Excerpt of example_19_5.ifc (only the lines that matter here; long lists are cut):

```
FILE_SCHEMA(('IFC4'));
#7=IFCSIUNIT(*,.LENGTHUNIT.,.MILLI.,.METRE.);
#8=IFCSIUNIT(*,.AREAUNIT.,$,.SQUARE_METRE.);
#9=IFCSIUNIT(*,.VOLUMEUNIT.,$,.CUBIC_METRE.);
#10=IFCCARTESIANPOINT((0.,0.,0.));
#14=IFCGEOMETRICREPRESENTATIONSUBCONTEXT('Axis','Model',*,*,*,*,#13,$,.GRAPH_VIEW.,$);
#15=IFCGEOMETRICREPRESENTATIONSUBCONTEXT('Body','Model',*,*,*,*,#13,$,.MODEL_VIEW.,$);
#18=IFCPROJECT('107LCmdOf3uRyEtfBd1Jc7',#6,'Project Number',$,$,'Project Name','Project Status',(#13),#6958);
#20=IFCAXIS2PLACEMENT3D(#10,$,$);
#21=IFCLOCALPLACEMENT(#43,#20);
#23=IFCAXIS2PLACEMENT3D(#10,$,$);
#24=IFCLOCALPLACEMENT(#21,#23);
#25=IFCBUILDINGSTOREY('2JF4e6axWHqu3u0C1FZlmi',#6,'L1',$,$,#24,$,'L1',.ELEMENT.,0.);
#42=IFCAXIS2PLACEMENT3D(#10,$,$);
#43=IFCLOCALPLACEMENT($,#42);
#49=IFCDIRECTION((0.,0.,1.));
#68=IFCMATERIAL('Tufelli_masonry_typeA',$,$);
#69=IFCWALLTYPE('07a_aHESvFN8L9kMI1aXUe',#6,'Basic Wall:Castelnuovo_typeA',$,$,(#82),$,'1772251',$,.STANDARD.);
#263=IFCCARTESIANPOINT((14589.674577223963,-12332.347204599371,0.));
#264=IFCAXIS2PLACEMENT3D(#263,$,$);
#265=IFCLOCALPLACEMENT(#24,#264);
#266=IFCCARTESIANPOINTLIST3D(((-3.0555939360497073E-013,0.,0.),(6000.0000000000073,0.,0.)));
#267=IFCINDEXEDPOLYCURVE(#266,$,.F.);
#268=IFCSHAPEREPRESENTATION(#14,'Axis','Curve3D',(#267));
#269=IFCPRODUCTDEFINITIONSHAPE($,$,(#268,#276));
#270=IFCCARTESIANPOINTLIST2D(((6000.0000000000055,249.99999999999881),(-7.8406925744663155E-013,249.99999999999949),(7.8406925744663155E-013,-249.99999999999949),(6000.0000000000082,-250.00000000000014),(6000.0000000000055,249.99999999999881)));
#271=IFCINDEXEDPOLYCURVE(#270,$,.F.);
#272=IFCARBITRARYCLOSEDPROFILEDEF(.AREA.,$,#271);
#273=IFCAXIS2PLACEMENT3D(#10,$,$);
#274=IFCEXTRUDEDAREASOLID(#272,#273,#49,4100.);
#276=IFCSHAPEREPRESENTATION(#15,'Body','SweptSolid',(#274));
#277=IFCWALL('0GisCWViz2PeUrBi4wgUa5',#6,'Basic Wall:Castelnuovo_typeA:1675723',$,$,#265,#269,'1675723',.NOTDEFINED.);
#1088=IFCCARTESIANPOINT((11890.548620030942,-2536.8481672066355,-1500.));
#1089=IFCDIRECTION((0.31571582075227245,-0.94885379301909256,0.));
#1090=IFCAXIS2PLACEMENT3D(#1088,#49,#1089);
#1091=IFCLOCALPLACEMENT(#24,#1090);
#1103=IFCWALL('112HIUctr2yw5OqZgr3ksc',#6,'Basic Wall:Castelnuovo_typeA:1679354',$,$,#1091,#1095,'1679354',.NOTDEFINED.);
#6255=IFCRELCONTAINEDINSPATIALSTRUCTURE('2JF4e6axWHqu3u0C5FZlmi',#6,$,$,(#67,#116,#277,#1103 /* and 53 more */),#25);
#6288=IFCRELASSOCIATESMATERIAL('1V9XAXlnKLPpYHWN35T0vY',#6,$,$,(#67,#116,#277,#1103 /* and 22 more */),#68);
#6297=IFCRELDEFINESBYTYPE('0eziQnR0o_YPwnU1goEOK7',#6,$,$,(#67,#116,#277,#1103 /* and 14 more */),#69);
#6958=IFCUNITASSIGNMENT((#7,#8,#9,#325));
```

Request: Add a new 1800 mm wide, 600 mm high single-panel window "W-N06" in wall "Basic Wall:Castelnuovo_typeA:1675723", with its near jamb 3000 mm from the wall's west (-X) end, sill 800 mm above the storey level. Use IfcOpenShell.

```python
import numpy as np
import ifcopenshell
import ifcopenshell.api.feature
import ifcopenshell.api.geometry
import ifcopenshell.api.root
import ifcopenshell.api.spatial
import ifcopenshell.geom
import ifcopenshell.util.element
import ifcopenshell.util.placement
import ifcopenshell.util.representation
import ifcopenshell.util.shape
import ifcopenshell.util.unit

model = ifcopenshell.open("example_19_5.ifc")
unit_scale = ifcopenshell.util.unit.calculate_unit_scale(model)
settings = ifcopenshell.geom.settings()


def volume(element):
    """Net volume in cubic metres, openings subtracted."""
    shape = ifcopenshell.geom.create_shape(settings, element)
    return ifcopenshell.util.shape.get_volume(shape.geometry)


wall = model.by_guid("0GisCWViz2PeUrBi4wgUa5")
storey = ifcopenshell.util.element.get_container(wall, ifc_class="IfcBuildingStorey")
context = ifcopenshell.util.representation.get_context(model, "Model", "Body", "MODEL_VIEW")
before = volume(wall)

width, height, from_end, sill = 1.8, 0.6, 3, 0.8  # metres

# The wall runs along its own X axis, and the end named is its -X end.
wall_shape = ifcopenshell.geom.create_shape(settings, wall)
x, y, z = ifcopenshell.util.shape.get_vertices(wall_shape.geometry).T
start = x.min() + from_end
face, thickness = float(y.min()), float(y.max() - y.min())
wall_matrix = ifcopenshell.util.placement.get_local_placement(wall.ObjectPlacement)
level = ifcopenshell.util.placement.get_local_placement(storey.ObjectPlacement)[2, 3]


def in_wall(x, y):
    """Placement at x, y metres in the wall's axes, at sill height."""
    matrix = wall_matrix.copy()
    matrix[:, 3] = wall_matrix @ np.array([x / unit_scale, y / unit_scale, 0.0, 1.0])
    matrix[2, 3] = level + sill / unit_scale
    return matrix


# Opening: a box that overshoots both wall faces by 50 mm.
opening = ifcopenshell.api.root.create_entity(model, ifc_class="IfcOpeningElement", predefined_type="OPENING")
box = ifcopenshell.api.geometry.add_wall_representation(
    model, context=context, length=width, height=height, thickness=thickness + 0.1
)
ifcopenshell.api.geometry.assign_representation(model, product=opening, representation=box)
ifcopenshell.api.geometry.edit_object_placement(model, product=opening, matrix=in_wall(start, face - 0.05), is_si=False)
ifcopenshell.api.feature.add_feature(model, feature=opening, element=wall)

window = ifcopenshell.api.root.create_entity(model, ifc_class="IfcWindow", name="W-N06", predefined_type="WINDOW")
window.OverallWidth, window.OverallHeight = width / unit_scale, height / unit_scale
window.PartitioningType = "SINGLE_PANEL"
body = ifcopenshell.api.geometry.add_window_representation(
    model,
    context=context,
    overall_width=window.OverallWidth,
    overall_height=window.OverallHeight,
    partition_type="SINGLE_PANEL",
)
ifcopenshell.api.geometry.assign_representation(model, product=window, representation=body)
ifcopenshell.api.spatial.assign_container(model, products=[window], relating_structure=storey)
ifcopenshell.api.feature.add_filling(model, opening=opening, element=window)

# Centre the window in the wall's thickness.
ifcopenshell.api.geometry.edit_object_placement(model, product=window, matrix=in_wall(start, face), is_si=False)
window_shape = ifcopenshell.geom.create_shape(settings, window)
depth = ifcopenshell.util.shape.get_vertices(window_shape.geometry)[:, 1]
offset = face + thickness / 2 - (depth.min() + depth.max()) / 2
ifcopenshell.api.geometry.edit_object_placement(model, product=window, matrix=in_wall(start, offset), is_si=False)

after = volume(wall)

print(f"wall volume {before:.3f} -> {after:.3f} m3")

model.write("example_19_5_edited.ifc")
```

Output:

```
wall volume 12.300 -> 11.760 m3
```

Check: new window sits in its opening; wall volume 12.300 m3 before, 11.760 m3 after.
